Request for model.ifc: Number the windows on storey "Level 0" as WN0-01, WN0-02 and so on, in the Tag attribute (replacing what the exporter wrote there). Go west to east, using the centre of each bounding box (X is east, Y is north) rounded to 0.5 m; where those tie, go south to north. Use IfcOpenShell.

First a look at what the model holds.

```python
import ifcopenshell
import ifcopenshell.util.element
import ifcopenshell.util.placement

model = ifcopenshell.open("model.ifc")
print(model.schema)
storey = next(s for s in model.by_type("IfcBuildingStorey") if s.Name == "Level 0")
windows = [e for e in ifcopenshell.util.element.get_decomposition(storey) if e.is_a("IfcWindow")]
for e in sorted(windows, key=lambda e: e.id()):
    origin = ifcopenshell.util.placement.get_local_placement(e.ObjectPlacement)[:3, 3]
    print(e.id(), e.Tag, e.Name, origin.round(2) + 0.0, sep=" | ")
```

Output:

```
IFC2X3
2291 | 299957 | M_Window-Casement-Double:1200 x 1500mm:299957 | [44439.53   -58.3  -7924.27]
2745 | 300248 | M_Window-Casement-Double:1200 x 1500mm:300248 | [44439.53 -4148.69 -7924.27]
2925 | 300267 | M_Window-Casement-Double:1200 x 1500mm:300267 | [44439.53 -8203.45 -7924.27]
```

```python
import ifcopenshell
import ifcopenshell.geom
import ifcopenshell.util.element
import ifcopenshell.util.shape

model = ifcopenshell.open("model.ifc")
settings = ifcopenshell.geom.settings()
settings.set("use-world-coords", True)


def centre(element):
    shape = ifcopenshell.geom.create_shape(settings, element)
    return ifcopenshell.util.shape.get_bbox_centroid(shape.geometry)


storey = next(s for s in model.by_type("IfcBuildingStorey") if s.Name == "Level 0")
windows = [e for e in ifcopenshell.util.element.get_decomposition(storey) if e.is_a("IfcWindow")]

# Insertion points can sit at a corner or the storey origin, so sort by the geometry (in metres).
centres = {e: centre(e) for e in windows}
windows.sort(key=lambda e: (round(centres[e][0] / 0.5), centres[e][1]))

for i, e in enumerate(windows, start=1):
    number = f"WN0-{i:02d}"
    e.Tag = number
    print(e.id(), number)

model.write("model_edited.ifc")
```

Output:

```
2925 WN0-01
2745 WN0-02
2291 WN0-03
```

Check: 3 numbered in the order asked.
